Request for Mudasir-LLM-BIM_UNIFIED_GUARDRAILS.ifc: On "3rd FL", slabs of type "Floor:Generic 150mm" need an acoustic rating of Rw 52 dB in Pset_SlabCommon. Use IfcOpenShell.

First a look at what the model holds.

```python
import ifcopenshell
import ifcopenshell.util.element

model = ifcopenshell.open("Mudasir-LLM-BIM_UNIFIED_GUARDRAILS.ifc")
print(model.schema)
storey = next(s for s in model.by_type("IfcBuildingStorey") if s.Name == "3rd FL")
slabs = [e for e in ifcopenshell.util.element.get_decomposition(storey) if e.is_a("IfcSlab")]
seen = {}
for e in slabs:
    element_type = ifcopenshell.util.element.get_type(e)
    key = (element_type.Name if element_type != e and element_type else None, ifcopenshell.util.element.get_pset(e, "Pset_SlabCommon", "AcousticRating"))
    seen[key] = seen.get(key, 0) + 1
for (name, value), count in sorted(seen.items(), key=str):
    print(count, "x", name, "|", value)
```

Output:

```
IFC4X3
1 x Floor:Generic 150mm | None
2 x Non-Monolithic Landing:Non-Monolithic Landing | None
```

```python
import ifcopenshell
import ifcopenshell.api.pset
import ifcopenshell.util.element

model = ifcopenshell.open("Mudasir-LLM-BIM_UNIFIED_GUARDRAILS.ifc")

storey = next(s for s in model.by_type("IfcBuildingStorey") if s.Name == "3rd FL")
slabs = [e for e in ifcopenshell.util.element.get_decomposition(storey) if e.is_a("IfcSlab")]

count = 0
for e in slabs:
    element_type = ifcopenshell.util.element.get_type(e)
    if element_type in (None, e) or element_type.Name != "Floor:Generic 150mm":
        continue
    # add_pset returns the element's existing set when there is one.
    pset = ifcopenshell.api.pset.add_pset(model, product=e, name="Pset_SlabCommon")
    ifcopenshell.api.pset.edit_pset(model, pset=pset, properties={"AcousticRating": "Rw 52 dB"})
    count += 1

print(count, "slabs updated")

model.write("Mudasir-LLM-BIM_UNIFIED_GUARDRAILS-out.ifc")
```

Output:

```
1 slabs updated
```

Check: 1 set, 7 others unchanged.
